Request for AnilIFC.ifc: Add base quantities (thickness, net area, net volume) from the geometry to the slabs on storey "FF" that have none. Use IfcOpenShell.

First a look at what the model holds.

```python
import ifcopenshell
import ifcopenshell.util.element
import ifcopenshell.util.unit

model = ifcopenshell.open("AnilIFC.ifc")
print(model.schema)
for unit_type in ("LENGTHUNIT", "AREAUNIT", "VOLUMEUNIT"):
    print(unit_type, ifcopenshell.util.unit.calculate_unit_scale(model, unit_type))
storey = next(s for s in model.by_type("IfcBuildingStorey") if s.Name == "FF")
slabs = [e for e in ifcopenshell.util.element.get_decomposition(storey) if e.is_a("IfcSlab")]
for e in sorted(slabs, key=lambda e: e.id()):
    print(e.id(), e.is_a(), e.Name, list(ifcopenshell.util.element.get_psets(e, qtos_only=True)), sep=" | ")
```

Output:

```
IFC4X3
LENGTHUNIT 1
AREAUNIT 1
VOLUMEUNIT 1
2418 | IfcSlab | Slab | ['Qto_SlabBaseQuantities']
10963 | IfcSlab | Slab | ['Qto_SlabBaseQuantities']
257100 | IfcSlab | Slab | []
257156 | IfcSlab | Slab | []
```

```python
import ifcopenshell
import ifcopenshell.api.pset
import ifcopenshell.geom
import ifcopenshell.util.element
import ifcopenshell.util.shape
import ifcopenshell.util.unit

model = ifcopenshell.open("AnilIFC.ifc")
unit_scale = ifcopenshell.util.unit.calculate_unit_scale(model)
area_scale = ifcopenshell.util.unit.calculate_unit_scale(model, "AREAUNIT")
volume_scale = ifcopenshell.util.unit.calculate_unit_scale(model, "VOLUMEUNIT")
settings = ifcopenshell.geom.settings()

storey = next(s for s in model.by_type("IfcBuildingStorey") if s.Name == "FF")
slabs = [e for e in ifcopenshell.util.element.get_decomposition(storey) if e.is_a("IfcSlab")]

for e in sorted(slabs, key=lambda e: e.id()):
    if ifcopenshell.util.element.get_psets(e, qtos_only=True, should_inherit=False):
        continue
    # Geometry comes back in metres, in the element's own axes.
    shape = ifcopenshell.geom.create_shape(settings, e)
    values = {
        "Width": ifcopenshell.util.shape.get_z(shape.geometry) / unit_scale,
        "NetArea": ifcopenshell.util.shape.get_footprint_area(shape.geometry) / area_scale,
        "NetVolume": ifcopenshell.util.shape.get_volume(shape.geometry) / volume_scale,
    }
    qto = ifcopenshell.api.pset.add_qto(model, product=e, name="Qto_SlabBaseQuantities")
    ifcopenshell.api.pset.edit_qto(model, qto=qto, properties=values)
    print(e.id(), {k: round(v, 3) for k, v in values.items()})

model.write("AnilIFC_v2.ifc")
```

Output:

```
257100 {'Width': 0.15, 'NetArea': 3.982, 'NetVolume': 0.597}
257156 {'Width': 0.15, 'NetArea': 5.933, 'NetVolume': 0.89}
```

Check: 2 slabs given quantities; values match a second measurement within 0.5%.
